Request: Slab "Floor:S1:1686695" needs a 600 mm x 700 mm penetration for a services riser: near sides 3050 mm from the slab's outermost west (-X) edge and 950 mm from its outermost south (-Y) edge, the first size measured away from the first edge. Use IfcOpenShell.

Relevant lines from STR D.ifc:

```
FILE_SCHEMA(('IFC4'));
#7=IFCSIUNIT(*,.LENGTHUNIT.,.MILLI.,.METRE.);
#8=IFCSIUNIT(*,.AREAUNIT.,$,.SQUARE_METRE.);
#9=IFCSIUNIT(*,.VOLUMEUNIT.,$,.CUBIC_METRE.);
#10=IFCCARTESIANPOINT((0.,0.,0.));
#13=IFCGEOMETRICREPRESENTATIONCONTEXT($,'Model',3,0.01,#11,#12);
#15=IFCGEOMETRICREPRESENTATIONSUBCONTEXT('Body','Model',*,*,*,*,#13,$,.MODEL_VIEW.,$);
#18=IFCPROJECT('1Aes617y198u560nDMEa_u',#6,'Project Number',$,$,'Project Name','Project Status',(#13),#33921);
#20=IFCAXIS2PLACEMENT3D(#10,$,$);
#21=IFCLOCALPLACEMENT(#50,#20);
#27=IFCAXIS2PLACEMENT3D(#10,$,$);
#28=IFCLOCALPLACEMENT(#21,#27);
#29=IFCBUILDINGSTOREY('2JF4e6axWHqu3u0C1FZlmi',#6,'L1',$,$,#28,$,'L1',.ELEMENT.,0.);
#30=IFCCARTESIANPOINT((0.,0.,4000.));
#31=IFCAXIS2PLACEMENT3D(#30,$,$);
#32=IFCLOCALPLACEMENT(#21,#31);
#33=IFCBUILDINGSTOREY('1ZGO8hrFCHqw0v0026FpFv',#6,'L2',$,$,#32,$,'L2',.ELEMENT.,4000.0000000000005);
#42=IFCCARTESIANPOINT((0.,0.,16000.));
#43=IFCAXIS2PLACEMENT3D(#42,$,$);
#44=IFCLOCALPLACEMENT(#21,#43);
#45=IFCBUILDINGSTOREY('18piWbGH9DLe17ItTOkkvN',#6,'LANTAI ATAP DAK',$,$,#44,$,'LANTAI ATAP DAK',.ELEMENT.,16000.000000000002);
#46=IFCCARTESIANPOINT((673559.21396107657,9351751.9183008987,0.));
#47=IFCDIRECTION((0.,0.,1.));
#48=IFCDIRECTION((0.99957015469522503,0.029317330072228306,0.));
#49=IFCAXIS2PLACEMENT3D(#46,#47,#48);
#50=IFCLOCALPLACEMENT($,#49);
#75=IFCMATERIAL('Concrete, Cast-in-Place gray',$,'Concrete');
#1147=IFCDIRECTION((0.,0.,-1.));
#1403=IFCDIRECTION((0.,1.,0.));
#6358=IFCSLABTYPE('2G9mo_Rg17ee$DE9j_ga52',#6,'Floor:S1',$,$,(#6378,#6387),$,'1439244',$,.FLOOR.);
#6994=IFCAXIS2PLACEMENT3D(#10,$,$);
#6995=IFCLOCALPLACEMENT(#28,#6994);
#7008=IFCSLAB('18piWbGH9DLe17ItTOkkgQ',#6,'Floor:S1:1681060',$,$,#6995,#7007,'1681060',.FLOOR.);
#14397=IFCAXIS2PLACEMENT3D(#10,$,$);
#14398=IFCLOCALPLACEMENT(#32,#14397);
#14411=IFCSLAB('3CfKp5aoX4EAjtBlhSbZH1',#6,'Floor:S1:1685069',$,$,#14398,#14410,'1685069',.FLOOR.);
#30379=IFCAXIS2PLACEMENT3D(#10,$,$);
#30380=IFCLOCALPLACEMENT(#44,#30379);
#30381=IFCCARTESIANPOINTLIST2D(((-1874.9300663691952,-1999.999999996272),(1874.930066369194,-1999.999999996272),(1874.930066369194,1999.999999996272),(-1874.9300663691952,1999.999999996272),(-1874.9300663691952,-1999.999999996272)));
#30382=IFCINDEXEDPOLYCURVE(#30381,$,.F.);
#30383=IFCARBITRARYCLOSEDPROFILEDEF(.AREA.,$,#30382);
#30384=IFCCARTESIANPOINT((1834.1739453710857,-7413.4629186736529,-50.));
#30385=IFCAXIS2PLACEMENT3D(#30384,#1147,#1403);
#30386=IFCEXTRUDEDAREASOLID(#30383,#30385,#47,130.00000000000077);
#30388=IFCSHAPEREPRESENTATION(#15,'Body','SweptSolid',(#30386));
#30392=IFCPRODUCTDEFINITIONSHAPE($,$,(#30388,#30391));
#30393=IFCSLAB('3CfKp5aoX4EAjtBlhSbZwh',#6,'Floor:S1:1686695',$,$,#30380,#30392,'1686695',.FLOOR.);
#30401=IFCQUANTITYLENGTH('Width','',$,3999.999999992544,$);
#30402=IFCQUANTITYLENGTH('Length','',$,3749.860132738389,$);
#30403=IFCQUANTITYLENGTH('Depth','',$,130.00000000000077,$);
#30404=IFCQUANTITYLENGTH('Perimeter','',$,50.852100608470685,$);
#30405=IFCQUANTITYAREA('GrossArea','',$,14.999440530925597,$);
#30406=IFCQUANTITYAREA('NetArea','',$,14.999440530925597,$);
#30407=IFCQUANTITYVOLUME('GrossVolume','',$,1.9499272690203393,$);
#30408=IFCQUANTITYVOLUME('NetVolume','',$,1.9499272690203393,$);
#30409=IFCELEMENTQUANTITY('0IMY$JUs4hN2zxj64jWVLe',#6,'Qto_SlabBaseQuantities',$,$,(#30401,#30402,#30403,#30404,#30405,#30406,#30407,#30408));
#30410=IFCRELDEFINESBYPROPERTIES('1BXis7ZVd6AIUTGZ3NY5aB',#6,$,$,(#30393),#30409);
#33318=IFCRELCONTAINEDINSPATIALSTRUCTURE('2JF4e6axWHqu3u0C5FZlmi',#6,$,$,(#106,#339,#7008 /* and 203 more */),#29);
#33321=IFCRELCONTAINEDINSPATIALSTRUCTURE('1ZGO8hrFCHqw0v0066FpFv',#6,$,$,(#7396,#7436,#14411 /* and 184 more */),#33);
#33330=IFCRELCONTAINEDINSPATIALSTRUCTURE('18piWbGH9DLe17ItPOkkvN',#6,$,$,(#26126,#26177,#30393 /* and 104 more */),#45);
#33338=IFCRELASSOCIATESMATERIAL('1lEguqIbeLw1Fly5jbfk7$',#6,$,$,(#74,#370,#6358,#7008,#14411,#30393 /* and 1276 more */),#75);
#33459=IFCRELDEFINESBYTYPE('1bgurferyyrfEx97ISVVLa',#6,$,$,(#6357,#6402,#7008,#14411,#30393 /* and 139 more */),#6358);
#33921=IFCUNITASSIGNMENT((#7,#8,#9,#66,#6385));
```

```python
import numpy as np
import ifcopenshell
import ifcopenshell.api.feature
import ifcopenshell.api.geometry
import ifcopenshell.api.pset
import ifcopenshell.api.root
import ifcopenshell.geom
import ifcopenshell.util.element
import ifcopenshell.util.placement
import ifcopenshell.util.representation
import ifcopenshell.util.shape
import ifcopenshell.util.unit

model = ifcopenshell.open("STR D.ifc")
unit_scale = ifcopenshell.util.unit.calculate_unit_scale(model)
area_scale = ifcopenshell.util.unit.calculate_unit_scale(model, "AREAUNIT")
volume_scale = ifcopenshell.util.unit.calculate_unit_scale(model, "VOLUMEUNIT")
settings = ifcopenshell.geom.settings()


def volume(element):
    """Net volume in cubic metres, openings subtracted."""
    shape = ifcopenshell.geom.create_shape(settings, element)
    return ifcopenshell.util.shape.get_volume(shape.geometry)


slab = model.by_guid("3CfKp5aoX4EAjtBlhSbZwh")
before = volume(slab)

# Extent in the slab's own axes, in metres. The edges named are its -X and -Y sides.
slab_shape = ifcopenshell.geom.create_shape(settings, slab)
vertices = ifcopenshell.util.shape.get_vertices(slab_shape.geometry)
x_min, y_min, bottom = vertices.min(axis=0)
top = vertices[:, 2].max()

opening = ifcopenshell.api.root.create_entity(model, ifc_class="IfcOpeningElement", name="Services riser opening", predefined_type="OPENING")
context = ifcopenshell.util.representation.get_context(model, "Model", "Body", "MODEL_VIEW")
width, depth = 0.6, 0.7
outline = [(0.0, 0.0), (width, 0.0), (width, depth), (0.0, depth), (0.0, 0.0)]
# Overshoot both faces by 50 mm so the cut is clean.
shape = ifcopenshell.api.geometry.add_slab_representation(
    model, context=context, depth=top - bottom + 0.1, polyline=outline
)
ifcopenshell.api.geometry.assign_representation(model, product=opening, representation=shape)

matrix = ifcopenshell.util.placement.get_local_placement(slab.ObjectPlacement)
matrix[:, 3] = matrix @ np.append(np.array([x_min + 3.05, y_min + 0.95, bottom - 0.05]) / unit_scale, 1.0)
ifcopenshell.api.geometry.edit_object_placement(model, product=opening, matrix=matrix, is_si=False)
ifcopenshell.api.feature.add_feature(model, feature=opening, element=slab)

after = volume(slab)

# Update the slab's stored quantities.
qto = model.by_id(ifcopenshell.util.element.get_pset(slab, "Qto_SlabBaseQuantities", should_inherit=False)["id"])
ifcopenshell.api.pset.edit_qto(model, qto=qto, properties={
    "NetArea": after / (top - bottom) / area_scale,
    "NetVolume": after / volume_scale,
})

print(f"slab volume {before:.3f} -> {after:.3f} m3")

model.write("STR D_v2.ifc")
```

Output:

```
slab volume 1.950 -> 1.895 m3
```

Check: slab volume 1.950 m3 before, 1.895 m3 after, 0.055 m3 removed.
